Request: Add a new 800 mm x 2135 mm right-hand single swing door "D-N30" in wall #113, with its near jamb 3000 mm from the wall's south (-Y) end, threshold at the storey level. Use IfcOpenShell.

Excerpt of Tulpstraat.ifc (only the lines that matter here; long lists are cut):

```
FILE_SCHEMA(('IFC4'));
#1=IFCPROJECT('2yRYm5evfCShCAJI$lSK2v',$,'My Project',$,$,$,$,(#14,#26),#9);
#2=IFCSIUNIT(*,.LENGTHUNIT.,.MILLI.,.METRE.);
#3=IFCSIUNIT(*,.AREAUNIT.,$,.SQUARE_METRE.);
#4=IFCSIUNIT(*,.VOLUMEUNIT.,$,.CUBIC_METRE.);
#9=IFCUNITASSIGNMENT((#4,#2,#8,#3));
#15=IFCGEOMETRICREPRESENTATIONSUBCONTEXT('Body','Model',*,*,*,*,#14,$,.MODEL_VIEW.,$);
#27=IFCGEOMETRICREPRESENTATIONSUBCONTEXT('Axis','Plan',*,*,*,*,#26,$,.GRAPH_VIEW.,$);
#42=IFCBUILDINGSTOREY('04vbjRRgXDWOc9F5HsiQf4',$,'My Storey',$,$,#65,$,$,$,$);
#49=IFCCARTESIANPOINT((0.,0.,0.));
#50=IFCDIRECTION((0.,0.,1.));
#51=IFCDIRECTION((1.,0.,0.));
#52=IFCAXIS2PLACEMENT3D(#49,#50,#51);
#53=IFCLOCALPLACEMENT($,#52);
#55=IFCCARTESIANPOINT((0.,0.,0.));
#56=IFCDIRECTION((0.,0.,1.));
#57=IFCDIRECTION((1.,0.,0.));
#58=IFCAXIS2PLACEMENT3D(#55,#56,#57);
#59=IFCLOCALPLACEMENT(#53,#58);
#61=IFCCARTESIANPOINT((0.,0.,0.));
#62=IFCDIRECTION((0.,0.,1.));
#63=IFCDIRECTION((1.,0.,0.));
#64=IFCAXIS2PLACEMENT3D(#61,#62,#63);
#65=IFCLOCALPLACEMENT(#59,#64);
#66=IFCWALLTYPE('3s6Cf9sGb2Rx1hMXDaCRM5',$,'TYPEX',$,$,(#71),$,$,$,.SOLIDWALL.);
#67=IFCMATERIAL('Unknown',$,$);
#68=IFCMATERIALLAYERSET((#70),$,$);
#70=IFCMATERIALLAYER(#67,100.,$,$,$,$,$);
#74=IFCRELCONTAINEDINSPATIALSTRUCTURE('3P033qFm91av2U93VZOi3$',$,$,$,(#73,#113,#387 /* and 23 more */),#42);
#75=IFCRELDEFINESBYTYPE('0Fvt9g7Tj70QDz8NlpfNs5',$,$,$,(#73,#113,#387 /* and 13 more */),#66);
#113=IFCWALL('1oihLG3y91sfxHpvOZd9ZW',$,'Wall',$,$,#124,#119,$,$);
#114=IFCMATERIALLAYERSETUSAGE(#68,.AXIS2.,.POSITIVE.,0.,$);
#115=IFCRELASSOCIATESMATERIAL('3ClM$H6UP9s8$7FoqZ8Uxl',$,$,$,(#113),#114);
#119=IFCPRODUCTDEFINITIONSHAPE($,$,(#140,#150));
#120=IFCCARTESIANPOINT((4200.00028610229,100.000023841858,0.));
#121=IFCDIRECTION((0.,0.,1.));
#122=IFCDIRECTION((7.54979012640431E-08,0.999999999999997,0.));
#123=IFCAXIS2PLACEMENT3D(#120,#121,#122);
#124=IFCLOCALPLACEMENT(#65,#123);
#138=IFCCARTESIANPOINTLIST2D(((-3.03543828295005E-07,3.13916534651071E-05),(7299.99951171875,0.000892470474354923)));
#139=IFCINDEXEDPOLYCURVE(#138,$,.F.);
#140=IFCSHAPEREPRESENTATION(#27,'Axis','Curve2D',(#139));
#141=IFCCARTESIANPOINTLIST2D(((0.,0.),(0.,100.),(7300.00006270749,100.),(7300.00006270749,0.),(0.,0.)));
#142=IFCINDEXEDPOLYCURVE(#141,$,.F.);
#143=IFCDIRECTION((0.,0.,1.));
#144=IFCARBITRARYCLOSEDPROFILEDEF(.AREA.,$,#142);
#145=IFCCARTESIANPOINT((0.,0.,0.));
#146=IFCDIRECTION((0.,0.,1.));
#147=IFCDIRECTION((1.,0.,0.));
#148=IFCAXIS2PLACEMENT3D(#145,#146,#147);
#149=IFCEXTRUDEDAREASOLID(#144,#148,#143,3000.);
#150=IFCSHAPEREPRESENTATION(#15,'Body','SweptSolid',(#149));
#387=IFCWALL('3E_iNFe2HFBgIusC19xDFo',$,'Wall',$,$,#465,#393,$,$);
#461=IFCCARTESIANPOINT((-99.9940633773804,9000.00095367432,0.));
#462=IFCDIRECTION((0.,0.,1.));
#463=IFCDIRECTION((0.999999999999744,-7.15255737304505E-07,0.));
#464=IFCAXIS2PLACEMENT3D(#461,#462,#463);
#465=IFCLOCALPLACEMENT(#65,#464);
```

```python
import numpy as np
import ifcopenshell
import ifcopenshell.api.feature
import ifcopenshell.api.geometry
import ifcopenshell.api.root
import ifcopenshell.api.spatial
import ifcopenshell.geom
import ifcopenshell.util.element
import ifcopenshell.util.placement
import ifcopenshell.util.representation
import ifcopenshell.util.shape
import ifcopenshell.util.unit

model = ifcopenshell.open("Tulpstraat.ifc")
unit_scale = ifcopenshell.util.unit.calculate_unit_scale(model)
settings = ifcopenshell.geom.settings()


def volume(element):
    """Net volume in cubic metres, openings subtracted."""
    shape = ifcopenshell.geom.create_shape(settings, element)
    return ifcopenshell.util.shape.get_volume(shape.geometry)


wall = model.by_guid("1oihLG3y91sfxHpvOZd9ZW")
storey = ifcopenshell.util.element.get_container(wall, ifc_class="IfcBuildingStorey")
context = ifcopenshell.util.representation.get_context(model, "Model", "Body", "MODEL_VIEW")
before = volume(wall)

width, height, from_end, sill = 0.8, 2.135, 3, 0.0  # metres

# The wall runs along its own X axis, and the end named is its -X end.
wall_shape = ifcopenshell.geom.create_shape(settings, wall)
x, y, z = ifcopenshell.util.shape.get_vertices(wall_shape.geometry).T
start = x.min() + from_end
face, thickness = float(y.min()), float(y.max() - y.min())
wall_matrix = ifcopenshell.util.placement.get_local_placement(wall.ObjectPlacement)
level = ifcopenshell.util.placement.get_local_placement(storey.ObjectPlacement)[2, 3]


def in_wall(x, y):
    """Placement at x, y metres in the wall's axes, at sill height."""
    matrix = wall_matrix.copy()
    matrix[:, 3] = wall_matrix @ np.array([x / unit_scale, y / unit_scale, 0.0, 1.0])
    matrix[2, 3] = level + sill / unit_scale
    return matrix


# Opening: a box that overshoots both wall faces by 50 mm.
opening = ifcopenshell.api.root.create_entity(model, ifc_class="IfcOpeningElement", predefined_type="OPENING")
box = ifcopenshell.api.geometry.add_wall_representation(
    model, context=context, length=width, height=height, thickness=thickness + 0.1
)
ifcopenshell.api.geometry.assign_representation(model, product=opening, representation=box)
ifcopenshell.api.geometry.edit_object_placement(model, product=opening, matrix=in_wall(start, face - 0.05), is_si=False)
ifcopenshell.api.feature.add_feature(model, feature=opening, element=wall)

door = ifcopenshell.api.root.create_entity(model, ifc_class="IfcDoor", name="D-N30", predefined_type="DOOR")
door.OverallWidth, door.OverallHeight = width / unit_scale, height / unit_scale
door.OperationType = "SINGLE_SWING_RIGHT"
body = ifcopenshell.api.geometry.add_door_representation(
    model,
    context=context,
    overall_width=door.OverallWidth,
    overall_height=door.OverallHeight,
    operation_type="SINGLE_SWING_RIGHT",
    lining_properties={"LiningDepth": thickness / unit_scale, "ThresholdDepth": thickness / unit_scale},
)
ifcopenshell.api.geometry.assign_representation(model, product=door, representation=body)
ifcopenshell.api.spatial.assign_container(model, products=[door], relating_structure=storey)
ifcopenshell.api.feature.add_filling(model, opening=opening, element=door)

# The lining spans the wall, so the door starts at the wall face.
ifcopenshell.api.geometry.edit_object_placement(model, product=door, matrix=in_wall(start, face), is_si=False)

after = volume(wall)

print(f"wall volume {before:.3f} -> {after:.3f} m3")

model.write("Tulpstraat_edited.ifc")
```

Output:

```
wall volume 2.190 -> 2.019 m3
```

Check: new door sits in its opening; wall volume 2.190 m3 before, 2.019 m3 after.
